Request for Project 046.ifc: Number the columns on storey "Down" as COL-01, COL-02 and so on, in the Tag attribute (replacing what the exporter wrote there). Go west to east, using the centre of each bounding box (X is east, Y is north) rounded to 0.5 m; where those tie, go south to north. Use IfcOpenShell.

First a look at what the model holds.

```python
import ifcopenshell
import ifcopenshell.util.element
import ifcopenshell.util.placement

model = ifcopenshell.open("Project 046.ifc")
print(model.schema)
storey = next(s for s in model.by_type("IfcBuildingStorey") if s.Name == "Down")
columns = [e for e in ifcopenshell.util.element.get_decomposition(storey) if e.is_a("IfcColumn")]
for e in sorted(columns, key=lambda e: e.id()):
    origin = ifcopenshell.util.placement.get_local_placement(e.ObjectPlacement)[:3, 3]
    print(e.id(), e.Tag, e.Name, origin.round(2) + 0.0, sep=" | ")
```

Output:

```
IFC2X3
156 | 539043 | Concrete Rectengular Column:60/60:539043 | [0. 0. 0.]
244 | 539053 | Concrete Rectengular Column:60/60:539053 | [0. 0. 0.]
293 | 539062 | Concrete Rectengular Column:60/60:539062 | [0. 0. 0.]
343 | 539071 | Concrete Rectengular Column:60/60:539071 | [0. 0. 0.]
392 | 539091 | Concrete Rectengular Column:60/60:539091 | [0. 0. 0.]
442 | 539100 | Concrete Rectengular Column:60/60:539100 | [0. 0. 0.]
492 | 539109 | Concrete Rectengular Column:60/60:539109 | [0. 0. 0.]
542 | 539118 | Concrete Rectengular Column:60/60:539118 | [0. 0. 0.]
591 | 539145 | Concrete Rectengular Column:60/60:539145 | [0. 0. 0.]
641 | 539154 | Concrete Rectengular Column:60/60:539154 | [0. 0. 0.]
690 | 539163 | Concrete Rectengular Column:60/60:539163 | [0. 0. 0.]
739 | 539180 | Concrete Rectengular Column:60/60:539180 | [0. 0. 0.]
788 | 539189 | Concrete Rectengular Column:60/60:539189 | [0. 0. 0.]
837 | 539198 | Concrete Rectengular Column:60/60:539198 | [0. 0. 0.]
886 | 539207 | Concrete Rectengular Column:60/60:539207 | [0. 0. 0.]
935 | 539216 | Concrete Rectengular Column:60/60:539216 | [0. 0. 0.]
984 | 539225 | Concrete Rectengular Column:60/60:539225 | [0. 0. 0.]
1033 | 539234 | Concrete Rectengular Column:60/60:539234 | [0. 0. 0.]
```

```python
import ifcopenshell
import ifcopenshell.geom
import ifcopenshell.util.element
import ifcopenshell.util.shape

model = ifcopenshell.open("Project 046.ifc")
settings = ifcopenshell.geom.settings()
settings.set("use-world-coords", True)


def centre(element):
    shape = ifcopenshell.geom.create_shape(settings, element)
    return ifcopenshell.util.shape.get_bbox_centroid(shape.geometry)


storey = next(s for s in model.by_type("IfcBuildingStorey") if s.Name == "Down")
columns = [e for e in ifcopenshell.util.element.get_decomposition(storey) if e.is_a("IfcColumn")]

# Insertion points can sit at a corner or the storey origin, so sort by the geometry (in metres).
centres = {e: centre(e) for e in columns}
columns.sort(key=lambda e: (round(centres[e][0] / 0.5), centres[e][1]))

for i, e in enumerate(columns, start=1):
    number = f"COL-{i:02d}"
    e.Tag = number
    print(e.id(), number)

model.write("Project 046_updated.ifc")
```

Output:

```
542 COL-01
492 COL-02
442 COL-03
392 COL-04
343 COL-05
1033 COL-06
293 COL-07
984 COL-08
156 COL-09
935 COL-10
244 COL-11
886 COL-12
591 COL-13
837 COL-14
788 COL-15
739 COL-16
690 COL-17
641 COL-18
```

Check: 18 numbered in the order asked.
